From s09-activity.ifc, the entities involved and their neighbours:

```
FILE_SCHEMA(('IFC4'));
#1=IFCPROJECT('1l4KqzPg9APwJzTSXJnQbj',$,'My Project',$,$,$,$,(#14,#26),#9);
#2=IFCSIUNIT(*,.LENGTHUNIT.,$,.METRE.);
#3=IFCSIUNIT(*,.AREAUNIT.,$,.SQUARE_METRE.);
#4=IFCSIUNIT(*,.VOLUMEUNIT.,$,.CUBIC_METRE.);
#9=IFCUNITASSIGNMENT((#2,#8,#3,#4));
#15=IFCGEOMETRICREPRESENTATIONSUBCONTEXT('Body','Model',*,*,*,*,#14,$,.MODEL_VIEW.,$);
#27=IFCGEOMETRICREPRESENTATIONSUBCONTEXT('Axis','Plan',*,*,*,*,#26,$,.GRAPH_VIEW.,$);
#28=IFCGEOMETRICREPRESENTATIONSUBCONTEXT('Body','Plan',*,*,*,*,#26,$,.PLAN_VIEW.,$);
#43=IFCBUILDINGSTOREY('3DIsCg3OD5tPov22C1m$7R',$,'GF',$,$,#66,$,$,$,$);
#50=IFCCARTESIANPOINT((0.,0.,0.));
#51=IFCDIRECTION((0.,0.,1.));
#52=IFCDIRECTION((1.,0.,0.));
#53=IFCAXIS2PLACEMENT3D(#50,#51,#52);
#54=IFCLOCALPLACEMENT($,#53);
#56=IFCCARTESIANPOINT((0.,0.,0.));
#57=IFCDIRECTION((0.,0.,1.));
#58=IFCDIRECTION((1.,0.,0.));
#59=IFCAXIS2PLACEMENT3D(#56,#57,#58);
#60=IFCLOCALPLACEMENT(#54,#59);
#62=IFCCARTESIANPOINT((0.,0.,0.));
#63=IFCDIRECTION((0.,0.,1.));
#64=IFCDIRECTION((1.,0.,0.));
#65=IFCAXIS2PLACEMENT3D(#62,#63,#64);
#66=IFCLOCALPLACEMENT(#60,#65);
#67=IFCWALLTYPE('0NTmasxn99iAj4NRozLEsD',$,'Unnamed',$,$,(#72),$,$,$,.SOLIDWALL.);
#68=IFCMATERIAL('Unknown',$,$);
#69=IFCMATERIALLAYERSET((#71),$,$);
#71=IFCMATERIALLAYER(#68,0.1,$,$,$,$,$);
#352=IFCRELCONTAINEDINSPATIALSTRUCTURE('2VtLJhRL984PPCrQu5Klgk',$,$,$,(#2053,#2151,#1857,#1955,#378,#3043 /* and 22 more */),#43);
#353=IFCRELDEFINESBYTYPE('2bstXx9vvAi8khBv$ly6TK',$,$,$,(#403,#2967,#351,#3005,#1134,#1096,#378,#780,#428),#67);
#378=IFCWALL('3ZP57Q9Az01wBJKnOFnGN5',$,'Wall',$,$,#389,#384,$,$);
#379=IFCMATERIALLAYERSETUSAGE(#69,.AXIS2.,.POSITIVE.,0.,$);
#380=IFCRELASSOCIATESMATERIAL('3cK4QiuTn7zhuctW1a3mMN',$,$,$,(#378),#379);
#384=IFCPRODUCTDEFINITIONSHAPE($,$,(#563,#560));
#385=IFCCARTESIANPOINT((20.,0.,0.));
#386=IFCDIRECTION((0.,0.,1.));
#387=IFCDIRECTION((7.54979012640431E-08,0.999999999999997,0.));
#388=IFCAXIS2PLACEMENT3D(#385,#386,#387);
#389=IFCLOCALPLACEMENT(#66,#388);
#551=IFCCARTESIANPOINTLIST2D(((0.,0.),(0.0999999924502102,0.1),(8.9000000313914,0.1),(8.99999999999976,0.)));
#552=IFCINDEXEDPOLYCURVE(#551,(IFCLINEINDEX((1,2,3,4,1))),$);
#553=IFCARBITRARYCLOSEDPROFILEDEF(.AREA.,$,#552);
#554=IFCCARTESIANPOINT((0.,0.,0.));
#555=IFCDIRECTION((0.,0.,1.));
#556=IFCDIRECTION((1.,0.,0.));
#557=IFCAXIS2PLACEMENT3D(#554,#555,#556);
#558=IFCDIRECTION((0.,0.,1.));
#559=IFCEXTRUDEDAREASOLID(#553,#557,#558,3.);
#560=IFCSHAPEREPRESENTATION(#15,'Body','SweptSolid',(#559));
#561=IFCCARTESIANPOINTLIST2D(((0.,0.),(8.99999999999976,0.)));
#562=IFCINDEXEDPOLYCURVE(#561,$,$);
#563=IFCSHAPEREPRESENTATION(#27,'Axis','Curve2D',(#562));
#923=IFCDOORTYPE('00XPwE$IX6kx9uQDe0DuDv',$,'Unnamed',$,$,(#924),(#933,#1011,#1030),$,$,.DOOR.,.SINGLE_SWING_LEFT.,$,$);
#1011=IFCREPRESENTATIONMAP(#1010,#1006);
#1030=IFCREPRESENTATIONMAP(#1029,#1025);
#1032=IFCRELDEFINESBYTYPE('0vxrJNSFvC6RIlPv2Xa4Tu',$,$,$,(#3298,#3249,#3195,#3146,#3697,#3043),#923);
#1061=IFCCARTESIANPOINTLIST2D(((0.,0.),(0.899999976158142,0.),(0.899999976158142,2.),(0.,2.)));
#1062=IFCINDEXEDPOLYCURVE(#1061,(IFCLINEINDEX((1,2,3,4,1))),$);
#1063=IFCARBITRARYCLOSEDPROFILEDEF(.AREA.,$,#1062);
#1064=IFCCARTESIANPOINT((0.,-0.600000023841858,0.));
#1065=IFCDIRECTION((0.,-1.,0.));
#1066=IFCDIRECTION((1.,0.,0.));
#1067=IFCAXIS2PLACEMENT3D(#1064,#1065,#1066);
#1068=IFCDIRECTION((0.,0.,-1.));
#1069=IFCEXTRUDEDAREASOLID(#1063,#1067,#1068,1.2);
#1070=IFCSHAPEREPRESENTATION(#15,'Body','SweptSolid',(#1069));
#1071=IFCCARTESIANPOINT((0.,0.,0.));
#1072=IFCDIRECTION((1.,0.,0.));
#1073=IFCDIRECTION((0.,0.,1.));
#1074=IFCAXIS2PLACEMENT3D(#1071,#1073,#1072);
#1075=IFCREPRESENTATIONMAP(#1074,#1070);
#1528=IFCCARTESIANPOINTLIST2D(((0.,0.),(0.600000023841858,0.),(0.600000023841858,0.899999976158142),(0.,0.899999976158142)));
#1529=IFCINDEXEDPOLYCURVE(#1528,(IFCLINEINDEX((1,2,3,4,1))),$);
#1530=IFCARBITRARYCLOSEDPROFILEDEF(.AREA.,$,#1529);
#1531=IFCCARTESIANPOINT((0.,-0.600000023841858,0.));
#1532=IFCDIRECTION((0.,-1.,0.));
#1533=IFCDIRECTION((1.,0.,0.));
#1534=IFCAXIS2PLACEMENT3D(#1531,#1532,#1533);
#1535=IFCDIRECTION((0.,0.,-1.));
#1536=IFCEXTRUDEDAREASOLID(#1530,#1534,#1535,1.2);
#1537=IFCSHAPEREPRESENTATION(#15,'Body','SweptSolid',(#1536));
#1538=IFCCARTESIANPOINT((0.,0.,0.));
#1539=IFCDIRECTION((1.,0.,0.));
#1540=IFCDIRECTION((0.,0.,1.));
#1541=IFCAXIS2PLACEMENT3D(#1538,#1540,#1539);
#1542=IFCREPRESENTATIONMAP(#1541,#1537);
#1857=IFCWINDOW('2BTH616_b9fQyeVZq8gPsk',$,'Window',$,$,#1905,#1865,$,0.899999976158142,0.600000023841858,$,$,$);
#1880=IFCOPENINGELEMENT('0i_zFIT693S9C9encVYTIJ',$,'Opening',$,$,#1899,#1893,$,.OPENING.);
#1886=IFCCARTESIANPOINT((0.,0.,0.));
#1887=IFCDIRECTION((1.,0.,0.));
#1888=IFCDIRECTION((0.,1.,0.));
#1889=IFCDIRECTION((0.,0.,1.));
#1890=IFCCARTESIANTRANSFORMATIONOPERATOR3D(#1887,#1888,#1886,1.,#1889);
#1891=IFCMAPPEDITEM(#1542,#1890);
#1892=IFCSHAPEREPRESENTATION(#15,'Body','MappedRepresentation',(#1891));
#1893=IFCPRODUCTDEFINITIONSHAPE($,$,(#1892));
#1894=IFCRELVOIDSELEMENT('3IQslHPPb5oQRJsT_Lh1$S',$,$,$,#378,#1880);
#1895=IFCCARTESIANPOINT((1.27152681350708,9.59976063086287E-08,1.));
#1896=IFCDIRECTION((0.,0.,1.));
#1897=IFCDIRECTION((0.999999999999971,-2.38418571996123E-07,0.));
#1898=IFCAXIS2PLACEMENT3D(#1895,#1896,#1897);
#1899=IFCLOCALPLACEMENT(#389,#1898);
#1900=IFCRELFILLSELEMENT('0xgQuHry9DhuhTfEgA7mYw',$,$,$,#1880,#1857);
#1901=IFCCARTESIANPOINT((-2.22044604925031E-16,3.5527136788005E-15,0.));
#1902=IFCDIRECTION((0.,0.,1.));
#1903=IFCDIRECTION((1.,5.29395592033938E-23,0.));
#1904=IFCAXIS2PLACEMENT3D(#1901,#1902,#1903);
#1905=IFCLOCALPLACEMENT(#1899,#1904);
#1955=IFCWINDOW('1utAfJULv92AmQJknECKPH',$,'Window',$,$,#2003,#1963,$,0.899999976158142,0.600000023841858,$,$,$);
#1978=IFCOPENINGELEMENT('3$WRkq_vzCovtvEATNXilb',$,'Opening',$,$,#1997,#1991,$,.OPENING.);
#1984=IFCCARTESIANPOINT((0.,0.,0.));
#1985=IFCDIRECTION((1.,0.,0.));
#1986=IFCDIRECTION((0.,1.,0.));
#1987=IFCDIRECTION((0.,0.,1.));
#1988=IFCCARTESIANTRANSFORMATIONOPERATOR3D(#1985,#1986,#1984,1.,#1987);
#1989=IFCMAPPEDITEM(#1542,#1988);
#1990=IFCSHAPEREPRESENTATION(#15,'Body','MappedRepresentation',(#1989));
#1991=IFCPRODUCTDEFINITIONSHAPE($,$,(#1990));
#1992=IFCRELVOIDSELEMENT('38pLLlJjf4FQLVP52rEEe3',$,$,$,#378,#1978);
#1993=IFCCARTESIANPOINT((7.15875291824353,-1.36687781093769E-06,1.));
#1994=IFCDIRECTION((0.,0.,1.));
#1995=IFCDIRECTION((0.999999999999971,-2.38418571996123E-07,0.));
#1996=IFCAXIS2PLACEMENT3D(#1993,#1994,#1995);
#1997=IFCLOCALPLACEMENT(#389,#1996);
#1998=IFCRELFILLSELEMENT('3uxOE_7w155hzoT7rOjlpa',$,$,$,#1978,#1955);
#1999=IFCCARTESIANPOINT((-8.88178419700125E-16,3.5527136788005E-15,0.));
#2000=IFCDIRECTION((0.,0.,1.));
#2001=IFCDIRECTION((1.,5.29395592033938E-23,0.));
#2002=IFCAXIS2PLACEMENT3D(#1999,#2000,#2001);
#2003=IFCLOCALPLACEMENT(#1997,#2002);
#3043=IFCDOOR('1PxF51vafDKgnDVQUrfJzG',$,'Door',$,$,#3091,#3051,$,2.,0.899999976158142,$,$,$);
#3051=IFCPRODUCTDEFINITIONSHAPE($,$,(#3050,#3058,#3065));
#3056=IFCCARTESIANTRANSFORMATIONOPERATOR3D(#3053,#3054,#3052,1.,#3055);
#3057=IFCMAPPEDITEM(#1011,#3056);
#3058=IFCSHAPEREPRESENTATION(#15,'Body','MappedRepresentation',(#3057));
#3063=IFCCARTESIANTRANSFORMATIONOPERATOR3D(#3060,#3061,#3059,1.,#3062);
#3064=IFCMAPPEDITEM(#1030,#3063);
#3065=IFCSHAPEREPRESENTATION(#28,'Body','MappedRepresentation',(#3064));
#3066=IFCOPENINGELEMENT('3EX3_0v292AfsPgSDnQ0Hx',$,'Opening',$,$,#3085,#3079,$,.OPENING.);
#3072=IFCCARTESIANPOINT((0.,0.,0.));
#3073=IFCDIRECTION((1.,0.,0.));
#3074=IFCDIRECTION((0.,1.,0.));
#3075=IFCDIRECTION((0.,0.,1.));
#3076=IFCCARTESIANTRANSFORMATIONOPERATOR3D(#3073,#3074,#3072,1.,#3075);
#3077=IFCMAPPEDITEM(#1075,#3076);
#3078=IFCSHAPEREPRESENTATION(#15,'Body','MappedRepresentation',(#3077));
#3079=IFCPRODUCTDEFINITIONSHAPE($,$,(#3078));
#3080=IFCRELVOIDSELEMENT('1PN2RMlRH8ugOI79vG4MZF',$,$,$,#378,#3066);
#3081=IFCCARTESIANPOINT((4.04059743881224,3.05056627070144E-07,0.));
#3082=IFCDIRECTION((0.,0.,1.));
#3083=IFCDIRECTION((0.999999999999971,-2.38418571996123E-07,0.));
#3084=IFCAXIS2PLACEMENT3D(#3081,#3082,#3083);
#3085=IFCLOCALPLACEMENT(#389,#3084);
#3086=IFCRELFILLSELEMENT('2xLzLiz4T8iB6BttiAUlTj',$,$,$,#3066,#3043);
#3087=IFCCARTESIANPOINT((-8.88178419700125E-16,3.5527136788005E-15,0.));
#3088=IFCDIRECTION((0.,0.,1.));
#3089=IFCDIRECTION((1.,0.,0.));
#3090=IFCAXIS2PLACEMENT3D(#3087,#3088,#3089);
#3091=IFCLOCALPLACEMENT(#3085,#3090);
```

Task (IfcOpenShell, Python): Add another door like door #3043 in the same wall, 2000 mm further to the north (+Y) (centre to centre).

```python
import ifcopenshell
import ifcopenshell.api.feature
import ifcopenshell.api.geometry
import ifcopenshell.api.root
import ifcopenshell.geom
import ifcopenshell.util.element
import ifcopenshell.util.placement
import ifcopenshell.util.shape
import ifcopenshell.util.unit

model = ifcopenshell.open("s09-activity.ifc")
unit_scale = ifcopenshell.util.unit.calculate_unit_scale(model)
settings = ifcopenshell.geom.settings()


def volume(element):
    """Net volume in cubic metres, openings subtracted."""
    shape = ifcopenshell.geom.create_shape(settings, element)
    return ifcopenshell.util.shape.get_volume(shape.geometry)


door = model.by_guid("1PxF51vafDKgnDVQUrfJzG")
opening = door.FillsVoids[0].RelatingOpeningElement
wall = opening.VoidsElements[0].RelatingBuildingElement
before = volume(wall)
shift = ifcopenshell.util.placement.get_local_placement(wall.ObjectPlacement)[:3, 0] * 2 / unit_scale

# copy_class copies the void relationship, type, container and properties, but no geometry.
new_opening = ifcopenshell.api.root.copy_class(model, product=opening)
new_opening.Representation = ifcopenshell.util.element.copy_deep(
    model, opening.Representation, exclude=["IfcGeometricRepresentationContext", "IfcRepresentationMap"]
)
new_door = ifcopenshell.api.root.copy_class(model, product=door)
new_door.Representation = ifcopenshell.util.element.copy_deep(
    model, door.Representation, exclude=["IfcGeometricRepresentationContext", "IfcRepresentationMap"]
)
ifcopenshell.api.feature.add_filling(model, opening=new_opening, element=new_door)

for old, new in ((opening, new_opening), (door, new_door)):
    matrix = ifcopenshell.util.placement.get_local_placement(old.ObjectPlacement)
    matrix[:3, 3] += shift
    ifcopenshell.api.geometry.edit_object_placement(model, product=new, matrix=matrix, is_si=False)

after = volume(wall)

print(f"wall volume {before:.3f} -> {after:.3f} m3")

model.write("s09-activity-out.ifc")
```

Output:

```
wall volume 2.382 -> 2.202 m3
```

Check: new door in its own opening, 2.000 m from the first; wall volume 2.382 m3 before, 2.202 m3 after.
